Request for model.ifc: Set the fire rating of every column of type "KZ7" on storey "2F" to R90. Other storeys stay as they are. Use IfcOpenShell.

First a look at what the model holds.

```python
import ifcopenshell
import ifcopenshell.util.element

model = ifcopenshell.open("model.ifc")
print(model.schema)
storey = next(s for s in model.by_type("IfcBuildingStorey") if s.Name == "2F")
columns = [e for e in ifcopenshell.util.element.get_decomposition(storey) if e.is_a("IfcColumn")]
seen = {}
for e in columns:
    element_type = ifcopenshell.util.element.get_type(e)
    key = (element_type.Name if element_type != e and element_type else None, ifcopenshell.util.element.get_pset(e, "Pset_ColumnCommon", "FireRating"))
    seen[key] = seen.get(key, 0) + 1
for (name, value), count in sorted(seen.items(), key=str):
    print(count, "x", name, "|", value)
```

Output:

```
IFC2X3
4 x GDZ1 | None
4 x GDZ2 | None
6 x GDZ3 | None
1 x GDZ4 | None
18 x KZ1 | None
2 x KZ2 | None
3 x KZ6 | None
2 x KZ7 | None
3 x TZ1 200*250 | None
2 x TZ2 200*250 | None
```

```python
import ifcopenshell
import ifcopenshell.api.pset
import ifcopenshell.util.element

model = ifcopenshell.open("model.ifc")

storey = next(s for s in model.by_type("IfcBuildingStorey") if s.Name == "2F")
columns = [e for e in ifcopenshell.util.element.get_decomposition(storey) if e.is_a("IfcColumn")]

count = 0
for e in columns:
    element_type = ifcopenshell.util.element.get_type(e)
    if element_type in (None, e) or element_type.Name != "KZ7":
        continue
    # add_pset returns the element's existing set when there is one.
    pset = ifcopenshell.api.pset.add_pset(model, product=e, name="Pset_ColumnCommon")
    ifcopenshell.api.pset.edit_pset(model, pset=pset, properties={"FireRating": "R90"})
    count += 1

print(count, "columns updated")

model.write("model_updated.ifc")
```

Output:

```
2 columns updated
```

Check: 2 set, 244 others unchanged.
